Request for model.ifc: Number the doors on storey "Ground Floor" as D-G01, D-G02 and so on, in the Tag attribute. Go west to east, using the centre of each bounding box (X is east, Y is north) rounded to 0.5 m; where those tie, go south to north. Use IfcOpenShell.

First a look at what the model holds.

```python
import ifcopenshell
import ifcopenshell.util.element
import ifcopenshell.util.placement

model = ifcopenshell.open("model.ifc")
print(model.schema)
storey = next(s for s in model.by_type("IfcBuildingStorey") if s.Name == "Ground Floor")
doors = [e for e in ifcopenshell.util.element.get_decomposition(storey) if e.is_a("IfcDoor")]
for e in sorted(doors, key=lambda e: e.id()):
    origin = ifcopenshell.util.placement.get_local_placement(e.ObjectPlacement)[:3, 3]
    print(e.id(), e.Tag, e.Name, origin.round(2) + 0.0, sep=" | ")
```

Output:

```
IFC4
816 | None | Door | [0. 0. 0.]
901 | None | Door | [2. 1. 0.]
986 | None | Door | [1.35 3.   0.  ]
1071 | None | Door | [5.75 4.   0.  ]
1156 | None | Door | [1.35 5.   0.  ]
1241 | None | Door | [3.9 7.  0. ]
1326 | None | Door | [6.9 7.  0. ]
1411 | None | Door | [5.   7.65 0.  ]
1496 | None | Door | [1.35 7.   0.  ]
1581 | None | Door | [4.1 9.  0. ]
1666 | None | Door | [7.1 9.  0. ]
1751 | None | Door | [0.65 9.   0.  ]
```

```python
import ifcopenshell
import ifcopenshell.geom
import ifcopenshell.util.element
import ifcopenshell.util.shape

model = ifcopenshell.open("model.ifc")
settings = ifcopenshell.geom.settings()
settings.set("use-world-coords", True)


def centre(element):
    shape = ifcopenshell.geom.create_shape(settings, element)
    return ifcopenshell.util.shape.get_bbox_centroid(shape.geometry)


storey = next(s for s in model.by_type("IfcBuildingStorey") if s.Name == "Ground Floor")
doors = [e for e in ifcopenshell.util.element.get_decomposition(storey) if e.is_a("IfcDoor")]

# Insertion points can sit at a corner or the storey origin, so sort by the geometry (in metres).
centres = {e: centre(e) for e in doors}
doors.sort(key=lambda e: (round(centres[e][0] / 0.5), centres[e][1]))

for i, e in enumerate(doors, start=1):
    number = f"D-G{i:02d}"
    e.Tag = number
    print(e.id(), number)

model.write("model-out.ifc")
```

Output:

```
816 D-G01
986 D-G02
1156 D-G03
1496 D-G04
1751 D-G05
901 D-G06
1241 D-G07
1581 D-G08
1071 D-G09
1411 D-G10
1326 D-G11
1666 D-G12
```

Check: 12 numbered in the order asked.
